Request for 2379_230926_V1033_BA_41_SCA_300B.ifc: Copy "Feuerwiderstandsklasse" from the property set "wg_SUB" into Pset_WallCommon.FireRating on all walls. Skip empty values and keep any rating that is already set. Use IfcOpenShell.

First a look at what the model holds.

```python
import ifcopenshell
import ifcopenshell.util.element

model = ifcopenshell.open("2379_230926_V1033_BA_41_SCA_300B.ifc")
print(model.schema)
walls = model.by_type("IfcWall")
print(len(walls), "walls")
for e in walls[:8]:
    source = ifcopenshell.util.element.get_pset(e, "wg_SUB", "Feuerwiderstandsklasse")
    target = ifcopenshell.util.element.get_pset(e, "Pset_WallCommon", "FireRating")
    print(e.id(), repr(source), repr(target), sep=" | ")
```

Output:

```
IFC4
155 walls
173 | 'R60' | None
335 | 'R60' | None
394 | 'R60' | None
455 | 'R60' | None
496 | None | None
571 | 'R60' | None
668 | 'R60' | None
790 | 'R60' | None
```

```python
import ifcopenshell
import ifcopenshell.api.pset
import ifcopenshell.util.element

model = ifcopenshell.open("2379_230926_V1033_BA_41_SCA_300B.ifc")

count = 0
for e in model.by_type("IfcWall"):
    value = ifcopenshell.util.element.get_pset(e, "wg_SUB", "Feuerwiderstandsklasse")
    current = ifcopenshell.util.element.get_pset(e, "Pset_WallCommon", "FireRating")
    if not value or not value.strip() or current:
        continue
    # add_pset returns the element's existing set when there is one.
    pset = ifcopenshell.api.pset.add_pset(model, product=e, name="Pset_WallCommon")
    ifcopenshell.api.pset.edit_pset(model, pset=pset, properties={"FireRating": value})
    count += 1

print(count, "walls updated")

model.write("2379_230926_V1033_BA_41_SCA_300B_updated.ifc")
```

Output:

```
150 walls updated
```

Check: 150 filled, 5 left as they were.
